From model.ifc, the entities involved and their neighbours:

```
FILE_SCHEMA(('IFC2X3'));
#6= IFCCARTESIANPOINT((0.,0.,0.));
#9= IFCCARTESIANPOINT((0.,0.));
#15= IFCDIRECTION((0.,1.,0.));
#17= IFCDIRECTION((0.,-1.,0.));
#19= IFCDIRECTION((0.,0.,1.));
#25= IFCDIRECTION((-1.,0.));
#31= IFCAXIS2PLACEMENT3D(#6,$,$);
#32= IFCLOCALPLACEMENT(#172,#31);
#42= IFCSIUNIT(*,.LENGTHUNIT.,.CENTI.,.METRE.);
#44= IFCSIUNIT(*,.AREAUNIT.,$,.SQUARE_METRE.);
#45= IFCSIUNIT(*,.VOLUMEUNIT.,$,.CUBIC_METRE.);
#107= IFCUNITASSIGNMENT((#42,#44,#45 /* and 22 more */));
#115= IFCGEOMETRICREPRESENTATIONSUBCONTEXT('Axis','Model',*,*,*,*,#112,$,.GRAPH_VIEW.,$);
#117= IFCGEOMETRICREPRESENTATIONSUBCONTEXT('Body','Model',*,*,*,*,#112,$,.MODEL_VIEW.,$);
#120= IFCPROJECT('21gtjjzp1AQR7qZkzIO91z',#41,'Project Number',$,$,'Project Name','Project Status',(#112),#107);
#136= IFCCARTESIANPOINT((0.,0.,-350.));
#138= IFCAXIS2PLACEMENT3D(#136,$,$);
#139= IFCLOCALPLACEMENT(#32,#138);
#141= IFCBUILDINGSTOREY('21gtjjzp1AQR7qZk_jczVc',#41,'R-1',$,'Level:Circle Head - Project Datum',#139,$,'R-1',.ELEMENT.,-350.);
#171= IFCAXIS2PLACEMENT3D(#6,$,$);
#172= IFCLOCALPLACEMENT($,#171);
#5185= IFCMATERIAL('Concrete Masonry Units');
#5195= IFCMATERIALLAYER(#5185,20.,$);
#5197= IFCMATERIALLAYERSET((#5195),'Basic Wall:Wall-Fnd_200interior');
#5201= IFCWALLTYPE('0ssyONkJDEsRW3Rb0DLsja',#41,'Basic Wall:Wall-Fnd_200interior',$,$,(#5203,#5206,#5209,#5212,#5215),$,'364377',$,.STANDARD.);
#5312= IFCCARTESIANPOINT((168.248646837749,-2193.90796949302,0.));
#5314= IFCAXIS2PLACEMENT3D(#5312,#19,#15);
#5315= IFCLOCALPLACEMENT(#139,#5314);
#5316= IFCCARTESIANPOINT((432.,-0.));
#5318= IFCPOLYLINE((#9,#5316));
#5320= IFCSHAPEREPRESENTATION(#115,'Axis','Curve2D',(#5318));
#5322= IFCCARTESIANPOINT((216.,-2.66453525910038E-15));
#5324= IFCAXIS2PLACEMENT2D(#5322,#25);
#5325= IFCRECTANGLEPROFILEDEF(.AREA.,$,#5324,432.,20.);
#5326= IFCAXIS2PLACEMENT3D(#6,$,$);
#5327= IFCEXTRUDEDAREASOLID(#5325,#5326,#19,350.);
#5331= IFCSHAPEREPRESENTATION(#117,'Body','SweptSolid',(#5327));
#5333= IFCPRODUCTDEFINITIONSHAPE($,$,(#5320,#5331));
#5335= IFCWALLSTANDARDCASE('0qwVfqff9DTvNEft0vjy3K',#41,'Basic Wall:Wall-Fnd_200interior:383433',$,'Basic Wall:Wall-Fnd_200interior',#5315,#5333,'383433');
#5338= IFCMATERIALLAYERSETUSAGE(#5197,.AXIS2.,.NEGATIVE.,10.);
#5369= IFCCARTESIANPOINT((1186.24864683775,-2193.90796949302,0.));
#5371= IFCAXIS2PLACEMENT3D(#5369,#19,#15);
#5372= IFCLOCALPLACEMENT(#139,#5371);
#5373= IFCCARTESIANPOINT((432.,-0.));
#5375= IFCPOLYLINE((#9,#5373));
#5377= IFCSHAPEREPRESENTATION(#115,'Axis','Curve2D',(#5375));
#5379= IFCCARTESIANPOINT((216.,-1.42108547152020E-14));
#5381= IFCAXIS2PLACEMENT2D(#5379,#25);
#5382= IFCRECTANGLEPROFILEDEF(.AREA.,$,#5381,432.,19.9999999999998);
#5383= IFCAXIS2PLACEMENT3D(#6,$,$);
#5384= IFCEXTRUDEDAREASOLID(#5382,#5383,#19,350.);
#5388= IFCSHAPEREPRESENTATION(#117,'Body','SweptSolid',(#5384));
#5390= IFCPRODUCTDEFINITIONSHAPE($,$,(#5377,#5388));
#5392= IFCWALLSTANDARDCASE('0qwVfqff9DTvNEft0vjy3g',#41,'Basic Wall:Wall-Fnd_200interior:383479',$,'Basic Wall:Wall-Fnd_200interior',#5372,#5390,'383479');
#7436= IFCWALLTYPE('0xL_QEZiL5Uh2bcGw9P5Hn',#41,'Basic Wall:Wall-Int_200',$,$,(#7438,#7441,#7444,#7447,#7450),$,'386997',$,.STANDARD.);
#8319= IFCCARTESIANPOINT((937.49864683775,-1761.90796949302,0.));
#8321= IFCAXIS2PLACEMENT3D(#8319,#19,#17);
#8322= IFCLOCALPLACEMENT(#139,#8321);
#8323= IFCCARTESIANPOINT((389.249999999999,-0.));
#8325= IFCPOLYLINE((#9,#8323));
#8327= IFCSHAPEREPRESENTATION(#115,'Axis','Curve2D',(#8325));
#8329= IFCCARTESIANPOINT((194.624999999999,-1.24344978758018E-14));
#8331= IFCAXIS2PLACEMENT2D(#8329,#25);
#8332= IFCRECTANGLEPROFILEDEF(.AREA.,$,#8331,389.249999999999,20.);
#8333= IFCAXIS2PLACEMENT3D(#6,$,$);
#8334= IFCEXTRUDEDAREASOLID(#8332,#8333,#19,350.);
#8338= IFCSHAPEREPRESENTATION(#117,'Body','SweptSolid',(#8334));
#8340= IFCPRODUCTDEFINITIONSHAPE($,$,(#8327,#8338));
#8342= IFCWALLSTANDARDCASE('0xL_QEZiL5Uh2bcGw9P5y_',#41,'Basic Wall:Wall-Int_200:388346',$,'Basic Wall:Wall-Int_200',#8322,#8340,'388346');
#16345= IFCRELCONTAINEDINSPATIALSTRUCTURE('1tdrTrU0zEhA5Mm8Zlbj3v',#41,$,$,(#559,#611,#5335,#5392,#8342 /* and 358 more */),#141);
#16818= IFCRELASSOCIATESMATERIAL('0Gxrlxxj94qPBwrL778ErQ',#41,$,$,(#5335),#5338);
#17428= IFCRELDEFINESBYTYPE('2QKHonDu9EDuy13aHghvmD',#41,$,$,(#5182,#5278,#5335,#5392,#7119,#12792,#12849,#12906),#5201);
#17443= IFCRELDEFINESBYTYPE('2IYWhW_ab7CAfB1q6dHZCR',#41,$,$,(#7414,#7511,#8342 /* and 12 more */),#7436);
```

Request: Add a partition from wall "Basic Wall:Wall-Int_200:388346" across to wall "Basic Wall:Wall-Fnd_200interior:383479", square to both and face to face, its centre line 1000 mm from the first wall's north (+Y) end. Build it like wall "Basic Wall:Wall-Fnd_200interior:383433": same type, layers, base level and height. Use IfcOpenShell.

```python
import numpy as np
import ifcopenshell
import ifcopenshell.api.geometry
import ifcopenshell.api.material
import ifcopenshell.api.pset
import ifcopenshell.api.root
import ifcopenshell.api.spatial
import ifcopenshell.api.type
import ifcopenshell.geom
import ifcopenshell.util.element
import ifcopenshell.util.placement
import ifcopenshell.util.representation
import ifcopenshell.util.shape
import ifcopenshell.util.unit

model = ifcopenshell.open("model.ifc")
unit_scale = ifcopenshell.util.unit.calculate_unit_scale(model)
settings = ifcopenshell.geom.settings()
settings.set("use-world-coords", True)

start_wall = model.by_guid("0xL_QEZiL5Uh2bcGw9P5y_")
end_wall = model.by_id(5392)
like = model.by_guid("0qwVfqff9DTvNEft0vjy3K")
matrix = ifcopenshell.util.placement.get_local_placement(start_wall.ObjectPlacement)
matrix[:3, 3] *= unit_scale


def extent(element):
    """Bounding box in the first wall's axes, in metres."""
    shape = ifcopenshell.geom.create_shape(settings, element)
    points = (ifcopenshell.util.shape.get_vertices(shape.geometry) - matrix[:3, 3]) @ matrix[:3, :3]
    return points.min(axis=0), points.max(axis=0)


y_start = extent(start_wall)[1][1]
y_end = extent(end_wall)[0][1]
like_min, like_max = extent(like)
length, height = float(abs(y_end - y_start)), float(like_max[2] - like_min[2])
layer_set = ifcopenshell.util.element.get_material(like, should_skip_usage=True)
thickness = sum(layer.LayerThickness for layer in layer_set.MaterialLayers) * unit_scale

wall = ifcopenshell.api.root.create_entity(model, ifc_class="IfcWallStandardCase", name="New partition")
storey = ifcopenshell.util.element.get_container(like)
ifcopenshell.api.spatial.assign_container(model, products=[wall], relating_structure=storey)
ifcopenshell.api.type.assign_type(
    model, related_objects=[wall], relating_type=ifcopenshell.util.element.get_type(like), should_map_representations=False
)
rel = ifcopenshell.api.material.assign_material(
    model, products=[wall], type="IfcMaterialLayerSetUsage", material=layer_set
)
rel.RelatingMaterial.OffsetFromReferenceLine = -thickness / 2 / unit_scale
pset = ifcopenshell.api.pset.add_pset(model, product=wall, name="Pset_WallCommon")
ifcopenshell.api.pset.edit_pset(model, pset=pset, properties={"IsExternal": False, "LoadBearing": False})

# The axis runs down the middle of the wall.
axis = ifcopenshell.api.geometry.add_axis_representation(
    model, context=ifcopenshell.util.representation.get_context(model, "Model", "Axis"), axis=[(0.0, 0.0), (length, 0.0)]
)
body = ifcopenshell.api.geometry.add_wall_representation(
    model,
    context=ifcopenshell.util.representation.get_context(model, "Model", "Body", "MODEL_VIEW"),
    length=length,
    height=height,
    thickness=thickness,
    offset=-thickness / 2,
)
for representation in (axis, body):
    ifcopenshell.api.geometry.assign_representation(model, product=wall, representation=representation)

placement = matrix @ ifcopenshell.util.placement.rotation(90, "Z")
placement[:, 3] = matrix @ np.array([extent(start_wall)[0][0] + 1, y_start, like_min[2], 1.0])
ifcopenshell.api.geometry.edit_object_placement(model, product=wall, matrix=placement)

print(f"partition {length:.3f} m long, {height:.3f} m high, {thickness:.3f} m thick")

model.write("model-out.ifc")
```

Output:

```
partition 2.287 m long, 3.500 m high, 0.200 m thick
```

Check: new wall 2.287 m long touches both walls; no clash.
